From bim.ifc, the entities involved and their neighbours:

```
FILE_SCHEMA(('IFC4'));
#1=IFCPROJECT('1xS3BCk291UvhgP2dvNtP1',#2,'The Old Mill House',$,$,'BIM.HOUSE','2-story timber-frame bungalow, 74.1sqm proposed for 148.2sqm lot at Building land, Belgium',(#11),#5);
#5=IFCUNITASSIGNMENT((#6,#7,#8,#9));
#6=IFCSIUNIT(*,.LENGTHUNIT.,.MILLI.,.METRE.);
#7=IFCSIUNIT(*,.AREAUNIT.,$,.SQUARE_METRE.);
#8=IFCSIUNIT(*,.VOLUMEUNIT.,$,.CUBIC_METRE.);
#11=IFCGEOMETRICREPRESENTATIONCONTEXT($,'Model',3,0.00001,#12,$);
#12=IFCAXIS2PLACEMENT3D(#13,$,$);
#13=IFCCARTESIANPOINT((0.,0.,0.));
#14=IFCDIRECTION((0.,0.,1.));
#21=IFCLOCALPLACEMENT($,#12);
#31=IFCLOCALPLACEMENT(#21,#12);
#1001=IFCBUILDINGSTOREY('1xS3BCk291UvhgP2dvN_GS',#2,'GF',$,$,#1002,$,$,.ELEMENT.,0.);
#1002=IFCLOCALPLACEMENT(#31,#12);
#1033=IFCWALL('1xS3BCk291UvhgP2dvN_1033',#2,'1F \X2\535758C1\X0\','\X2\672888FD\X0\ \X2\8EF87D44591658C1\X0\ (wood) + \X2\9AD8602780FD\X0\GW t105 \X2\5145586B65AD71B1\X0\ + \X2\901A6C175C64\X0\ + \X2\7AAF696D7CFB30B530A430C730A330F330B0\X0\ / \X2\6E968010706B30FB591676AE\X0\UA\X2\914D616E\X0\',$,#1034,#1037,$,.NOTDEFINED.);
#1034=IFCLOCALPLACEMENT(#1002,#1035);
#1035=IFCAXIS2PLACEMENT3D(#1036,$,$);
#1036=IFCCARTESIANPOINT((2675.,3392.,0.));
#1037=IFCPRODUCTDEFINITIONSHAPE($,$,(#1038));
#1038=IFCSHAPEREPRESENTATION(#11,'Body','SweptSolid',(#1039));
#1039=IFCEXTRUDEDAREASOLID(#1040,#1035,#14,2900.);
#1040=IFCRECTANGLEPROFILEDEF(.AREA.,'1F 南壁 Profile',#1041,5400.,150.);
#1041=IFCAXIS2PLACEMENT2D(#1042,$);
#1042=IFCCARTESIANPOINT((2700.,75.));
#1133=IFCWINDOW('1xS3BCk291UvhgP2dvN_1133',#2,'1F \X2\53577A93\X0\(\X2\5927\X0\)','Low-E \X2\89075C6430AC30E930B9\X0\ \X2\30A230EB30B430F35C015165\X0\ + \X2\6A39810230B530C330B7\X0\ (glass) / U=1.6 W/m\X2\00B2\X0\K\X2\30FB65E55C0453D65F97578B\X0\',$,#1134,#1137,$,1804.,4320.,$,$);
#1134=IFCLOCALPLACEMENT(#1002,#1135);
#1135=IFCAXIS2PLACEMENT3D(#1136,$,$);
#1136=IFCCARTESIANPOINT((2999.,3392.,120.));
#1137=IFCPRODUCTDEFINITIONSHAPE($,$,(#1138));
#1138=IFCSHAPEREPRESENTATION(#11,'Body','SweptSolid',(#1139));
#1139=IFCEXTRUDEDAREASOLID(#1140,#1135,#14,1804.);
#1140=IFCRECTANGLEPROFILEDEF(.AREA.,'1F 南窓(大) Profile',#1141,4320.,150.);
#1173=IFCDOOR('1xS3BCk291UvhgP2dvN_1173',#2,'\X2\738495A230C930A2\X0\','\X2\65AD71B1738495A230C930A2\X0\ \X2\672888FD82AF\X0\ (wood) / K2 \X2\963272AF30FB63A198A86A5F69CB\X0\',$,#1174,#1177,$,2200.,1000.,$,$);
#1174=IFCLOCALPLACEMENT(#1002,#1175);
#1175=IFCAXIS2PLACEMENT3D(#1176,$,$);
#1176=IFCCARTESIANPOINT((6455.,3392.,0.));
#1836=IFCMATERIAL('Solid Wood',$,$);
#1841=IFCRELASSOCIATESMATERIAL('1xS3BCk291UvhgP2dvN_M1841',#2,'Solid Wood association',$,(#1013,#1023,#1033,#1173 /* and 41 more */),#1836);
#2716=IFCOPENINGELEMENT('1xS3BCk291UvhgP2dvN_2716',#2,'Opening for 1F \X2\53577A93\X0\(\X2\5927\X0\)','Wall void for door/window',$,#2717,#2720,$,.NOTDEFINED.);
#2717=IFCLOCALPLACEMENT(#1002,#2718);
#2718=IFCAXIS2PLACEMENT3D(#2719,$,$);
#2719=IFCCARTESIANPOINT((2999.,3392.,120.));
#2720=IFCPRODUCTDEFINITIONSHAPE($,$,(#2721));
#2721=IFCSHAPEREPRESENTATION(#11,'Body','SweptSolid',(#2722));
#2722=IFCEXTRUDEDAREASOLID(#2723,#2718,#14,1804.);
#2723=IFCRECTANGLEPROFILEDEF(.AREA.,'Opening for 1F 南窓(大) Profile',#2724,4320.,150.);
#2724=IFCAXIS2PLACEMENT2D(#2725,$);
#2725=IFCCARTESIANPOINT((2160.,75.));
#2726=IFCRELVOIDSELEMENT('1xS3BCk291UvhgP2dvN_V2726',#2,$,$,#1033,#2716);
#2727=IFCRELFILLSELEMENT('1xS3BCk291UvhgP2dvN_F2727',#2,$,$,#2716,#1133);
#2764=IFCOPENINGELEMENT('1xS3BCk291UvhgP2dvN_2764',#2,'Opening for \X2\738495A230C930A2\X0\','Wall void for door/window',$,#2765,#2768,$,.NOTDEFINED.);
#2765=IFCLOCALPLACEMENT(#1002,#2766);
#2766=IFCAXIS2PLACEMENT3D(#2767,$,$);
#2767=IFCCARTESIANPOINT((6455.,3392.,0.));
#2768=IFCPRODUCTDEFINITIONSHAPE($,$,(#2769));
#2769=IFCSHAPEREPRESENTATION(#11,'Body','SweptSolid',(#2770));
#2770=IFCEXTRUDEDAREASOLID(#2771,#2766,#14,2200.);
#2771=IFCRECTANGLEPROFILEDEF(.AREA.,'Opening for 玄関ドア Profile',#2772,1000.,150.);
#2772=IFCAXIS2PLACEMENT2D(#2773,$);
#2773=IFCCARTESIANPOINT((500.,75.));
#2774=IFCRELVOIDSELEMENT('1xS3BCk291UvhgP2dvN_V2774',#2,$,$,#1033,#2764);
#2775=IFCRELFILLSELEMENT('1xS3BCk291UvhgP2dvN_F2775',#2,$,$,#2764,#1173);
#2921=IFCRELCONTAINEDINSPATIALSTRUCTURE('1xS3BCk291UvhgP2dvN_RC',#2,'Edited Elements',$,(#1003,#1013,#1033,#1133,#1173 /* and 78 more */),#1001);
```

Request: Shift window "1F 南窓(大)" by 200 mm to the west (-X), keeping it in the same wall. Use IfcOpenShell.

```python
import ifcopenshell
import ifcopenshell.api.geometry
import ifcopenshell.util.placement
import ifcopenshell.util.unit

model = ifcopenshell.open("bim.ifc")
unit_scale = ifcopenshell.util.unit.calculate_unit_scale(model)

window = model.by_guid("1xS3BCk291UvhgP2dvN_1133")
opening = window.FillsVoids[0].RelatingOpeningElement
wall = opening.VoidsElements[0].RelatingBuildingElement

wall_matrix = ifcopenshell.util.placement.get_local_placement(wall.ObjectPlacement)
shift = wall_matrix[:3, 0] * -0.2 / unit_scale
before = ifcopenshell.util.placement.get_local_placement(window.ObjectPlacement)[:3, 3].copy()

# The window is not placed relative to its opening, so move both.
for product in (opening, window):
    matrix = ifcopenshell.util.placement.get_local_placement(product.ObjectPlacement)
    matrix[:3, 3] += shift
    ifcopenshell.api.geometry.edit_object_placement(model, product=product, matrix=matrix, is_si=False)

after = ifcopenshell.util.placement.get_local_placement(window.ObjectPlacement)[:3, 3]
print("window moved by", (after - before).round(3) + 0.0)

model.write("bim_updated.ifc")
```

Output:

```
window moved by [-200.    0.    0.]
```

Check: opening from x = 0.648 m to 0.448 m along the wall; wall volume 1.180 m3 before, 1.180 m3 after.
